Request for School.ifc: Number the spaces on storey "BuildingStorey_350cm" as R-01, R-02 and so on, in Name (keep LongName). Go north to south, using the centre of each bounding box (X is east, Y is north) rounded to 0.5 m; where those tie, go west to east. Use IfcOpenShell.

First a look at what the model holds.

```python
import ifcopenshell
import ifcopenshell.util.element
import ifcopenshell.util.placement

model = ifcopenshell.open("School.ifc")
print(model.schema)
storey = next(s for s in model.by_type("IfcBuildingStorey") if s.Name == "BuildingStorey_350cm")
spaces = [e for e in ifcopenshell.util.element.get_decomposition(storey) if e.is_a("IfcSpace")]
for e in sorted(spaces, key=lambda e: e.id()):
    origin = ifcopenshell.util.placement.get_local_placement(e.ObjectPlacement)[:3, 3]
    print(e.id(), e.Name, e.LongName, origin.round(2) + 0.0, sep=" | ")
```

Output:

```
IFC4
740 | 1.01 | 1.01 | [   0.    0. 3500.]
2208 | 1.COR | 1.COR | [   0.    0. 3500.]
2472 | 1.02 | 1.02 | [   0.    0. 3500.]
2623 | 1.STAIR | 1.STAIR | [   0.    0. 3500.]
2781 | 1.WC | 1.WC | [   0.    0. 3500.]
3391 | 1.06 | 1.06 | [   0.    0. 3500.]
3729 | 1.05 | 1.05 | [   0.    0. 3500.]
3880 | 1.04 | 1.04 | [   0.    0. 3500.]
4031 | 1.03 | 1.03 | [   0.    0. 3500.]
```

```python
import ifcopenshell
import ifcopenshell.geom
import ifcopenshell.util.element
import ifcopenshell.util.shape

model = ifcopenshell.open("School.ifc")
settings = ifcopenshell.geom.settings()
settings.set("use-world-coords", True)


def centre(element):
    shape = ifcopenshell.geom.create_shape(settings, element)
    return ifcopenshell.util.shape.get_bbox_centroid(shape.geometry)


storey = next(s for s in model.by_type("IfcBuildingStorey") if s.Name == "BuildingStorey_350cm")
spaces = [e for e in ifcopenshell.util.element.get_decomposition(storey) if e.is_a("IfcSpace")]

# Insertion points can sit at a corner or the storey origin, so sort by the geometry (in metres).
centres = {e: centre(e) for e in spaces}
spaces.sort(key=lambda e: (-round(centres[e][1] / 0.5), centres[e][0]))

for i, e in enumerate(spaces, start=1):
    number = f"R-{i:02d}"
    e.Name = number
    print(e.id(), number)

model.write("School-out.ifc")
```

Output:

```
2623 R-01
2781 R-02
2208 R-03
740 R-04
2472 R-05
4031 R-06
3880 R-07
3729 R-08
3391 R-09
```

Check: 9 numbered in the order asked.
